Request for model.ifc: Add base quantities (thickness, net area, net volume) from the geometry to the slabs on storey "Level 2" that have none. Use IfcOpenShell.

First a look at what the model holds.

```python
import ifcopenshell
import ifcopenshell.util.element
import ifcopenshell.util.unit

model = ifcopenshell.open("model.ifc")
print(model.schema)
for unit_type in ("LENGTHUNIT", "AREAUNIT", "VOLUMEUNIT"):
    print(unit_type, ifcopenshell.util.unit.calculate_unit_scale(model, unit_type))
storey = next(s for s in model.by_type("IfcBuildingStorey") if s.Name == "Level 2")
slabs = [e for e in ifcopenshell.util.element.get_decomposition(storey) if e.is_a("IfcSlab")]
for e in sorted(slabs, key=lambda e: e.id()):
    print(e.id(), e.is_a(), e.Name, list(ifcopenshell.util.element.get_psets(e, qtos_only=True)), sep=" | ")
```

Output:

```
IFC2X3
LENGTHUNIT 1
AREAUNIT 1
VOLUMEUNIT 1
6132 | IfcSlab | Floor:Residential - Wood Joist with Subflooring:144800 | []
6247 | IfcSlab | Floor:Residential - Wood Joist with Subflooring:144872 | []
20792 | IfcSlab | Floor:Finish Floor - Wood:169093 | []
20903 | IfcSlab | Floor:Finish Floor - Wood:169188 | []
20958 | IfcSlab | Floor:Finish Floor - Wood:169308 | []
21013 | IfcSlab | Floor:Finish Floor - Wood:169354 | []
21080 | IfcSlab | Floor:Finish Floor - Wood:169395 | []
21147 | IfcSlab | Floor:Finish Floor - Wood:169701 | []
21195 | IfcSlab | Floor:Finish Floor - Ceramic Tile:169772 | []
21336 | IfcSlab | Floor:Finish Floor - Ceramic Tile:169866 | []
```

```python
import ifcopenshell
import ifcopenshell.api.pset
import ifcopenshell.geom
import ifcopenshell.util.element
import ifcopenshell.util.shape
import ifcopenshell.util.unit

model = ifcopenshell.open("model.ifc")
unit_scale = ifcopenshell.util.unit.calculate_unit_scale(model)
area_scale = ifcopenshell.util.unit.calculate_unit_scale(model, "AREAUNIT")
volume_scale = ifcopenshell.util.unit.calculate_unit_scale(model, "VOLUMEUNIT")
settings = ifcopenshell.geom.settings()

storey = next(s for s in model.by_type("IfcBuildingStorey") if s.Name == "Level 2")
slabs = [e for e in ifcopenshell.util.element.get_decomposition(storey) if e.is_a("IfcSlab")]

for e in sorted(slabs, key=lambda e: e.id()):
    if ifcopenshell.util.element.get_psets(e, qtos_only=True, should_inherit=False):
        continue
    # Geometry comes back in metres, in the element's own axes.
    shape = ifcopenshell.geom.create_shape(settings, e)
    values = {
        "Width": ifcopenshell.util.shape.get_z(shape.geometry) / unit_scale,
        "NetArea": ifcopenshell.util.shape.get_footprint_area(shape.geometry) / area_scale,
        "NetVolume": ifcopenshell.util.shape.get_volume(shape.geometry) / volume_scale,
    }
    qto = ifcopenshell.api.pset.add_qto(model, product=e, name="BaseQuantities")
    ifcopenshell.api.pset.edit_qto(model, qto=qto, properties=values)
    print(e.id(), {k: round(v, 3) for k, v in values.items()})

model.write("model_updated.ifc")
```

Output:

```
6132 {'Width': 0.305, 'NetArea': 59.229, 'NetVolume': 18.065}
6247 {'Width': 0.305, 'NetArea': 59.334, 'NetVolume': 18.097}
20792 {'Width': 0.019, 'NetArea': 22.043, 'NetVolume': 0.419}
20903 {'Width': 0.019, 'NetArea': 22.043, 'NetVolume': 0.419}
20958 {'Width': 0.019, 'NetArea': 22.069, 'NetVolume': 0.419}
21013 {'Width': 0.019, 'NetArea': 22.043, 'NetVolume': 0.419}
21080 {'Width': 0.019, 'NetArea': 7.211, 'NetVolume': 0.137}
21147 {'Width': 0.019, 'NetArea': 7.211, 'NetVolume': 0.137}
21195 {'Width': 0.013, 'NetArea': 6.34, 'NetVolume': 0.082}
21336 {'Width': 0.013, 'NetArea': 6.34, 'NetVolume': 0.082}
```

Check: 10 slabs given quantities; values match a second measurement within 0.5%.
